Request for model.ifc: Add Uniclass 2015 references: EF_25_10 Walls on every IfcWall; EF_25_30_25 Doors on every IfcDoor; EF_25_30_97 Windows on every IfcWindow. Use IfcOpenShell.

First a look at what the model holds.

```python
import ifcopenshell

model = ifcopenshell.open("model.ifc")
print(model.schema)
print("classifications:", [c.Name for c in model.by_type("IfcClassification")])
for ifc_class in ("IfcDoor", "IfcRoof", "IfcStair", "IfcWall", "IfcWindow"):
    print(ifc_class, len(model.by_type(ifc_class)))
```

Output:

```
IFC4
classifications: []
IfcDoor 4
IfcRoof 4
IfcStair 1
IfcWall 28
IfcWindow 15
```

```python
import ifcopenshell
import ifcopenshell.api.classification

model = ifcopenshell.open("model.ifc")

system = ifcopenshell.api.classification.add_classification(model, classification="Uniclass 2015")

codes = {
    "IfcWall": ("EF_25_10", "Walls"),
    "IfcDoor": ("EF_25_30_25", "Doors"),
    "IfcWindow": ("EF_25_30_97", "Windows"),
}
for ifc_class, (code, name) in codes.items():
    products = model.by_type(ifc_class)
    ifcopenshell.api.classification.add_reference(
        model, products=products, classification=system, identification=code, name=name
    )
    print(code, len(products))

model.write("model_rev.ifc")
```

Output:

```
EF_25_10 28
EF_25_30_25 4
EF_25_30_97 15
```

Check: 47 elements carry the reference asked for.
